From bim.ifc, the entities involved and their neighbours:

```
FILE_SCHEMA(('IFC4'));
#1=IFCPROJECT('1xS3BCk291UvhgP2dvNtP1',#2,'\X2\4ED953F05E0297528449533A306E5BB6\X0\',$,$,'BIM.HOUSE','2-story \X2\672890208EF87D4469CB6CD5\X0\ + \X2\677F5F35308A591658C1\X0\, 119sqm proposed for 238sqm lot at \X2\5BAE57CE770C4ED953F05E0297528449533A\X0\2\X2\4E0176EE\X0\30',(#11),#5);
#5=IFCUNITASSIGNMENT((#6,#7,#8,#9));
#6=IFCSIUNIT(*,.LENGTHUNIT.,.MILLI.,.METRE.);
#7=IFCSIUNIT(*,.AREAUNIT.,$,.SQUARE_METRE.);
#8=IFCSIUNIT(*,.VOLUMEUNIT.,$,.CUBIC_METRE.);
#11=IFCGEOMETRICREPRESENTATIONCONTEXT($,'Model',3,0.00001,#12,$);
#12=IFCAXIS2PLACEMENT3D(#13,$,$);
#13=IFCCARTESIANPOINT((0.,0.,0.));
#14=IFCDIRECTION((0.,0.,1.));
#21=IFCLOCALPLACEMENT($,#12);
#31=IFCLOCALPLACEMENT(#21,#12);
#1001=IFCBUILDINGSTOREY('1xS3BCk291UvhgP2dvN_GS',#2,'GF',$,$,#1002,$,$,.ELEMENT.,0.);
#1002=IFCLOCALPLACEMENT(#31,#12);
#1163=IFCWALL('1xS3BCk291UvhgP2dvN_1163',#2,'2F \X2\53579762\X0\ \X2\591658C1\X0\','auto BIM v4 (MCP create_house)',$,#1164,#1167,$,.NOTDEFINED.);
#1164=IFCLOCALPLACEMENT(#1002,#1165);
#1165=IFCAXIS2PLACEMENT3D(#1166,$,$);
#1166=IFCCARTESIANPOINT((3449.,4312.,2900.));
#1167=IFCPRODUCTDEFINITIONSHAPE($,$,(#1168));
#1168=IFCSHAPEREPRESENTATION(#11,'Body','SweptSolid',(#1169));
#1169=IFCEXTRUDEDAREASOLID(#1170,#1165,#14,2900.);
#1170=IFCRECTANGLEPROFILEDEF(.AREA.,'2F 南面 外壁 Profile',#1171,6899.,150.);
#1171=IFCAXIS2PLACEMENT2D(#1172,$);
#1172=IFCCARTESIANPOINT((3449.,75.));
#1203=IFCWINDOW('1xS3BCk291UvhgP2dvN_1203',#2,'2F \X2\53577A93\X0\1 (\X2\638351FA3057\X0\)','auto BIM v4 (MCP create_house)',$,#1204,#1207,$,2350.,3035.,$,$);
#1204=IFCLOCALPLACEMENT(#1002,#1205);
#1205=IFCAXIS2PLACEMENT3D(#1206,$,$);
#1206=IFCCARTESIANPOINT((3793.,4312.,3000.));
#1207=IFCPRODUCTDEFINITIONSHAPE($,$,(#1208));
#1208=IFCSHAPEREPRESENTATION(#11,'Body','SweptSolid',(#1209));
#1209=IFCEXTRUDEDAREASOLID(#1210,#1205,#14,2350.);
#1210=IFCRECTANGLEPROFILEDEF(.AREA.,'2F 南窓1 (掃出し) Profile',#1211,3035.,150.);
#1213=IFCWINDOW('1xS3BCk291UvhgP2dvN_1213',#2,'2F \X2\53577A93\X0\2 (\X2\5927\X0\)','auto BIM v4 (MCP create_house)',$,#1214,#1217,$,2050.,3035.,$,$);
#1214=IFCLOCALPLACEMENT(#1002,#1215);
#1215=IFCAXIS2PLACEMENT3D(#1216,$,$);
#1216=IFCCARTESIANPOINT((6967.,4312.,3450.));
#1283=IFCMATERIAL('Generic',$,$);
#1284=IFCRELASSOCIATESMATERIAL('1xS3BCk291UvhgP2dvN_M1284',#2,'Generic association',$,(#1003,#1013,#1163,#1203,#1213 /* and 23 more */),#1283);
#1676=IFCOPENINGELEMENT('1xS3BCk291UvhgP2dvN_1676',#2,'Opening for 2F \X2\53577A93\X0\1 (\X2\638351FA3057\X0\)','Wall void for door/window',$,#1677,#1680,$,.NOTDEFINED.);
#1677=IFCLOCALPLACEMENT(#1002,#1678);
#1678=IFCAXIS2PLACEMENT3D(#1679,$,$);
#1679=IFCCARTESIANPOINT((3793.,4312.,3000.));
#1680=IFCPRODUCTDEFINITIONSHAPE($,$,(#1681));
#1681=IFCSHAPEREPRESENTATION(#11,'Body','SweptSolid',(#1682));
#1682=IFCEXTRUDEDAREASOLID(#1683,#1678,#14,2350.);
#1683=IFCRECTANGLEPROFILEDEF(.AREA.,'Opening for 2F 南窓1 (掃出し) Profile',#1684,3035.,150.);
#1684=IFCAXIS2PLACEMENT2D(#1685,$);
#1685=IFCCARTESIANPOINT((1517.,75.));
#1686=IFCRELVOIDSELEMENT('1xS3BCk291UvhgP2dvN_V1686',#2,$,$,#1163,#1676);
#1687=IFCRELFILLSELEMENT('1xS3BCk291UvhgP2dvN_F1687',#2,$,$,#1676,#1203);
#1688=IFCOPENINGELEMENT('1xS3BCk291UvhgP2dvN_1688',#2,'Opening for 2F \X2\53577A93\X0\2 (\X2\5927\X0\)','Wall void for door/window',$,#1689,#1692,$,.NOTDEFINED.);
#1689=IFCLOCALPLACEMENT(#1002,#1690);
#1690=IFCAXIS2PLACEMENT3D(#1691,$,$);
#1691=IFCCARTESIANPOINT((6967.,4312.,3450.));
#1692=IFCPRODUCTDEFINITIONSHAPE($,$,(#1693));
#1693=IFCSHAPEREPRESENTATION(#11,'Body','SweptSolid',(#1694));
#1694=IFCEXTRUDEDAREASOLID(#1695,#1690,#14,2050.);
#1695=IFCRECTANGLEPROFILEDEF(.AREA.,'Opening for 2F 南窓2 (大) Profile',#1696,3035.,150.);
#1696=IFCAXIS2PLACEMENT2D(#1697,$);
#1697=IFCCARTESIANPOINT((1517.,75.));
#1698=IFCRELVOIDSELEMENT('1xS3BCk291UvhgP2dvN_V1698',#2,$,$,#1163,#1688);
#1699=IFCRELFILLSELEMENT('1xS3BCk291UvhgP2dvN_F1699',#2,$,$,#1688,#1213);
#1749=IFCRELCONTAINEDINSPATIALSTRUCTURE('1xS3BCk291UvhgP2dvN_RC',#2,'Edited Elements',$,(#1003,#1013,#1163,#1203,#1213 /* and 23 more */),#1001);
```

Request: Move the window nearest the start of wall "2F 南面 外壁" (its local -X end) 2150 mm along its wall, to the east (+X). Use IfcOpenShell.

```python
import ifcopenshell
import ifcopenshell.api.geometry
import ifcopenshell.util.placement

model = ifcopenshell.open("bim.ifc")

window = model.by_guid("1xS3BCk291UvhgP2dvN_1203")
opening = window.FillsVoids[0].RelatingOpeningElement
wall = opening.VoidsElements[0].RelatingBuildingElement

wall_matrix = ifcopenshell.util.placement.get_local_placement(wall.ObjectPlacement)
shift = wall_matrix[:3, 0] * 2150.0
before = ifcopenshell.util.placement.get_local_placement(window.ObjectPlacement)[:3, 3].copy()

# The window is not placed relative to its opening, so move both.
for product in (opening, window):
    matrix = ifcopenshell.util.placement.get_local_placement(product.ObjectPlacement)
    matrix[:3, 3] += shift
    ifcopenshell.api.geometry.edit_object_placement(model, product=product, matrix=matrix, is_si=False)

after = ifcopenshell.util.placement.get_local_placement(window.ObjectPlacement)[:3, 3]
print("window moved by", (after - before).round(3) + 0.0)

model.write("bim_rev.ifc")
```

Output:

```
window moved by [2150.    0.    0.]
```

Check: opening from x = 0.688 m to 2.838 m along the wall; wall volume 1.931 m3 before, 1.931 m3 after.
